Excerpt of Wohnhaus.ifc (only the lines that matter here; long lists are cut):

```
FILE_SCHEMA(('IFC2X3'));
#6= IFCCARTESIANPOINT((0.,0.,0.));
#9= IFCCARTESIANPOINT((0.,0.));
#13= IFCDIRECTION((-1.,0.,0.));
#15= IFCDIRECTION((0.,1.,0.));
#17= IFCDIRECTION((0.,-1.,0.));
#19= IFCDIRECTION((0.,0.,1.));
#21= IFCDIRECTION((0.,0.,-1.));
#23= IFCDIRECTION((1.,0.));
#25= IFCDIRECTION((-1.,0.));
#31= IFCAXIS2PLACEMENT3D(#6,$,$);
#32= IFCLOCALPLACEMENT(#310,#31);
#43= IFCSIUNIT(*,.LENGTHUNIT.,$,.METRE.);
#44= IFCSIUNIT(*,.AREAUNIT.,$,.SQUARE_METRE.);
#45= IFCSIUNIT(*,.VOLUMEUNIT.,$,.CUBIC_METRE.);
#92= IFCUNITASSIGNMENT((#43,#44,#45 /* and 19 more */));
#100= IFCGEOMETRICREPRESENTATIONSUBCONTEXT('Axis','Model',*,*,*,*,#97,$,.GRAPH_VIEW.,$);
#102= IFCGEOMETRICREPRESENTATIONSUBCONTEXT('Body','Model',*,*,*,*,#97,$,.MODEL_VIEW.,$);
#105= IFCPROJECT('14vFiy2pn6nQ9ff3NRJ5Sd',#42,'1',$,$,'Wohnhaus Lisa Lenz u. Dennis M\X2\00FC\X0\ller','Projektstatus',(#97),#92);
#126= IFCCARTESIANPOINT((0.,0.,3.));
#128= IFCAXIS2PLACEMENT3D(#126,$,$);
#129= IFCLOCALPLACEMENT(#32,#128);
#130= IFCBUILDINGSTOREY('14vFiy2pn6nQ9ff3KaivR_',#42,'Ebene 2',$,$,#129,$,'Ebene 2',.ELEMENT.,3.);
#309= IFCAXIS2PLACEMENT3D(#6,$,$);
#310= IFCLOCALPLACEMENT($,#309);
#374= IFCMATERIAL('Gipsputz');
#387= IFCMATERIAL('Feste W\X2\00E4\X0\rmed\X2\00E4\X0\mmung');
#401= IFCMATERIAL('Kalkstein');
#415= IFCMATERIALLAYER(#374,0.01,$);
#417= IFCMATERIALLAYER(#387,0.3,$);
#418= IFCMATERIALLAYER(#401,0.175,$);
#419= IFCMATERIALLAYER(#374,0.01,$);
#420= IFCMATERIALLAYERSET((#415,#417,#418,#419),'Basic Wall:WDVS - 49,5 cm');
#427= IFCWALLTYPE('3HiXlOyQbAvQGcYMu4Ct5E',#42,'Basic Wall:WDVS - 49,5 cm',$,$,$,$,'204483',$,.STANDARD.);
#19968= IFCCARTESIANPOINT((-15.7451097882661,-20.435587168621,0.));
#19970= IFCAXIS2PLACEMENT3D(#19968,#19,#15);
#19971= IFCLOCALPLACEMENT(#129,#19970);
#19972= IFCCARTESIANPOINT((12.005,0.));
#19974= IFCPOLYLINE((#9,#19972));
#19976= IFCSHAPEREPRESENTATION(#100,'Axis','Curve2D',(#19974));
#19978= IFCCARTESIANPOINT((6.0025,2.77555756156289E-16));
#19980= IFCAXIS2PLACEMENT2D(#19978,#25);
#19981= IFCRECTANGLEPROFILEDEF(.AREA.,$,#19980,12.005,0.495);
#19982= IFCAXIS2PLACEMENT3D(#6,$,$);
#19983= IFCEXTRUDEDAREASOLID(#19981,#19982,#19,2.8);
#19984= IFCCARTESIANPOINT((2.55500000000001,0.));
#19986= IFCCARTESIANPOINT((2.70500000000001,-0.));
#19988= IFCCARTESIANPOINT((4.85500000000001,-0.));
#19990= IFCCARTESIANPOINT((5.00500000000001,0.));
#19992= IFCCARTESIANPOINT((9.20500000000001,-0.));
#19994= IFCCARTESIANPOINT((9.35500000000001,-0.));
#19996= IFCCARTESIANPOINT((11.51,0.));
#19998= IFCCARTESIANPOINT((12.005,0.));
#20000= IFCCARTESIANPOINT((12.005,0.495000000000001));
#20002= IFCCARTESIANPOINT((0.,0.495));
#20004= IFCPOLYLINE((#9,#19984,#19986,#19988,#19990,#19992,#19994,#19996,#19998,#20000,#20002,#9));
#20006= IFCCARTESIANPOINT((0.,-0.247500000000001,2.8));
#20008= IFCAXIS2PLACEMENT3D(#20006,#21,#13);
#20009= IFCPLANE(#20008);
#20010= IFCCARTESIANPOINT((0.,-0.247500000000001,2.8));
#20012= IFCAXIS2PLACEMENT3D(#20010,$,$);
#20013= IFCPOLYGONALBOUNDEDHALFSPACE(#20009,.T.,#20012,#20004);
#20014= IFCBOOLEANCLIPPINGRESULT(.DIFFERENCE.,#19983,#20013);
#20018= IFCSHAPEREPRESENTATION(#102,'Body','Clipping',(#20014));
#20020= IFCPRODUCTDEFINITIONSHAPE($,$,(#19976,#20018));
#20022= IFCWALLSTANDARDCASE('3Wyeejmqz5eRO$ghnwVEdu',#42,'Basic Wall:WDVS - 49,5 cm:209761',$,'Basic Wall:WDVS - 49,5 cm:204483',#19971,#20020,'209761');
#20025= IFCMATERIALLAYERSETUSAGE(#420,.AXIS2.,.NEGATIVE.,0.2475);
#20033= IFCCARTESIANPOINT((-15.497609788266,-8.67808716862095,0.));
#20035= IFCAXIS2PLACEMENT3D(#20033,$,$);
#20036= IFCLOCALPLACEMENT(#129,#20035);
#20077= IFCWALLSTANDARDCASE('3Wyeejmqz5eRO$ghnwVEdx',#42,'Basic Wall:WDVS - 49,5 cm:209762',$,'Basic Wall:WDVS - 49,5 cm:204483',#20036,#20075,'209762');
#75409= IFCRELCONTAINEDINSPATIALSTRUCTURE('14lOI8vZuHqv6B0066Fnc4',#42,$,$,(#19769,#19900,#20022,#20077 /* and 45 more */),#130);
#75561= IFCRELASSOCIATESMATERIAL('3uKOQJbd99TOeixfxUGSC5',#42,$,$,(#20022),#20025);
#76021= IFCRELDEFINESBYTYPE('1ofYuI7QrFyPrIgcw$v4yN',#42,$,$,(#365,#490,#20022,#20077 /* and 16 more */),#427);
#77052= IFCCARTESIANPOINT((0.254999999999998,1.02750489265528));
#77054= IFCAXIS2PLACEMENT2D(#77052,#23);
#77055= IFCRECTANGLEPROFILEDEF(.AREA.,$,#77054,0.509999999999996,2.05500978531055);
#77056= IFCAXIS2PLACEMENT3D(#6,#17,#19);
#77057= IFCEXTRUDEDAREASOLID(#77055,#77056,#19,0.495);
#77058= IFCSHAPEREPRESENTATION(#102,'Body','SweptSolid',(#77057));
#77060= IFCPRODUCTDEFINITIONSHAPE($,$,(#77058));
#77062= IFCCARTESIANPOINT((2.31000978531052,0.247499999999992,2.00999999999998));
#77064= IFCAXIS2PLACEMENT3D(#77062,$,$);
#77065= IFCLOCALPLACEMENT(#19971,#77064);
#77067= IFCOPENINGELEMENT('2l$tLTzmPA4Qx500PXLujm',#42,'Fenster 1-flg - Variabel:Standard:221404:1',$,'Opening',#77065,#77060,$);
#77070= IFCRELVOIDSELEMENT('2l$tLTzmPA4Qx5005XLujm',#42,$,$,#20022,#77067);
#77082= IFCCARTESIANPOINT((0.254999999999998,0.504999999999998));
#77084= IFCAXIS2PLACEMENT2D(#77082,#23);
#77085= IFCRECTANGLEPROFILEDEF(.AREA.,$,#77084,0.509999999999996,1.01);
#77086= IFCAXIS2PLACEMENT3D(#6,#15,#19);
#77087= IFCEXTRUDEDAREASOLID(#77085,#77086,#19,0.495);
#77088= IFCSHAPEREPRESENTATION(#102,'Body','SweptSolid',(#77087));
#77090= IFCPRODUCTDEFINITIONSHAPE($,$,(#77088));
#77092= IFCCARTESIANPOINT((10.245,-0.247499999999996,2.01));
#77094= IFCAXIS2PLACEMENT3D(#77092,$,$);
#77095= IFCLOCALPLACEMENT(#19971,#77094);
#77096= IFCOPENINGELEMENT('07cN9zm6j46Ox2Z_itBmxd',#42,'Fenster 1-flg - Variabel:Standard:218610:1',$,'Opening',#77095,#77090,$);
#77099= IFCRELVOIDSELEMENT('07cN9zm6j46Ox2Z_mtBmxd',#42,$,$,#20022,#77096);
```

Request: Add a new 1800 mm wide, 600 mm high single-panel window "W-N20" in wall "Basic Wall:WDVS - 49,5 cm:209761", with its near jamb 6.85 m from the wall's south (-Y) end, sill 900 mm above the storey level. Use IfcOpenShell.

```python
import numpy as np
import ifcopenshell
import ifcopenshell.api.feature
import ifcopenshell.api.geometry
import ifcopenshell.api.root
import ifcopenshell.api.spatial
import ifcopenshell.api.type
import ifcopenshell.geom
import ifcopenshell.util.element
import ifcopenshell.util.placement
import ifcopenshell.util.representation
import ifcopenshell.util.shape
import ifcopenshell.util.unit

model = ifcopenshell.open("Wohnhaus.ifc")
unit_scale = ifcopenshell.util.unit.calculate_unit_scale(model)
settings = ifcopenshell.geom.settings()


def volume(element):
    """Net volume in cubic metres, openings subtracted."""
    shape = ifcopenshell.geom.create_shape(settings, element)
    return ifcopenshell.util.shape.get_volume(shape.geometry)


wall = model.by_guid("3Wyeejmqz5eRO$ghnwVEdu")
storey = ifcopenshell.util.element.get_container(wall, ifc_class="IfcBuildingStorey")
context = ifcopenshell.util.representation.get_context(model, "Model", "Body", "MODEL_VIEW")
before = volume(wall)

width, height, from_end, sill = 1.8, 0.6, 6.85, 0.9  # metres

# The wall runs along its own X axis, and the end named is its -X end.
wall_shape = ifcopenshell.geom.create_shape(settings, wall)
x, y, z = ifcopenshell.util.shape.get_vertices(wall_shape.geometry).T
start = x.min() + from_end
face, thickness = float(y.min()), float(y.max() - y.min())
wall_matrix = ifcopenshell.util.placement.get_local_placement(wall.ObjectPlacement)
level = ifcopenshell.util.placement.get_local_placement(storey.ObjectPlacement)[2, 3]


def in_wall(x, y):
    """Placement at x, y metres in the wall's axes, at sill height."""
    matrix = wall_matrix.copy()
    matrix[:, 3] = wall_matrix @ np.array([x / unit_scale, y / unit_scale, 0.0, 1.0])
    matrix[2, 3] = level + sill / unit_scale
    return matrix


# Opening: a box that overshoots both wall faces by 50 mm.
opening = ifcopenshell.api.root.create_entity(model, ifc_class="IfcOpeningElement")
box = ifcopenshell.api.geometry.add_wall_representation(
    model, context=context, length=width, height=height, thickness=thickness + 0.1
)
ifcopenshell.api.geometry.assign_representation(model, product=opening, representation=box)
ifcopenshell.api.geometry.edit_object_placement(model, product=opening, matrix=in_wall(start, face - 0.05), is_si=False)
ifcopenshell.api.feature.add_feature(model, feature=opening, element=wall)

window = ifcopenshell.api.root.create_entity(model, ifc_class="IfcWindow", name="W-N20")
window.OverallWidth, window.OverallHeight = width / unit_scale, height / unit_scale
body = ifcopenshell.api.geometry.add_window_representation(
    model,
    context=context,
    overall_width=window.OverallWidth,
    overall_height=window.OverallHeight,
    partition_type="SINGLE_PANEL",
)
ifcopenshell.api.geometry.assign_representation(model, product=window, representation=body)
ifcopenshell.api.spatial.assign_container(model, products=[window], relating_structure=storey)
fills = ifcopenshell.api.feature.add_filling(model, opening=opening, element=window)
fills.OwnerHistory = window.OwnerHistory  # required in IFC2X3

# IFC2X3 keeps the operation on the window style.
style = ifcopenshell.api.root.create_entity(model, ifc_class="IfcWindowStyle", name="W-N20")
style.OperationType, style.ConstructionType = "SINGLE_PANEL", "NOTDEFINED"
style.ParameterTakesPrecedence = style.Sizeable = False
ifcopenshell.api.type.assign_type(model, related_objects=[window], relating_type=style)

# Centre the window in the wall's thickness.
ifcopenshell.api.geometry.edit_object_placement(model, product=window, matrix=in_wall(start, face), is_si=False)
window_shape = ifcopenshell.geom.create_shape(settings, window)
depth = ifcopenshell.util.shape.get_vertices(window_shape.geometry)[:, 1]
offset = face + thickness / 2 - (depth.min() + depth.max()) / 2
ifcopenshell.api.geometry.edit_object_placement(model, product=window, matrix=in_wall(start, offset), is_si=False)

after = volume(wall)

print(f"wall volume {before:.3f} -> {after:.3f} m3")

model.write("Wohnhaus-out.ifc")
```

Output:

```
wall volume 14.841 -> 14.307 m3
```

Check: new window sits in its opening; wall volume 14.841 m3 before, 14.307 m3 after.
